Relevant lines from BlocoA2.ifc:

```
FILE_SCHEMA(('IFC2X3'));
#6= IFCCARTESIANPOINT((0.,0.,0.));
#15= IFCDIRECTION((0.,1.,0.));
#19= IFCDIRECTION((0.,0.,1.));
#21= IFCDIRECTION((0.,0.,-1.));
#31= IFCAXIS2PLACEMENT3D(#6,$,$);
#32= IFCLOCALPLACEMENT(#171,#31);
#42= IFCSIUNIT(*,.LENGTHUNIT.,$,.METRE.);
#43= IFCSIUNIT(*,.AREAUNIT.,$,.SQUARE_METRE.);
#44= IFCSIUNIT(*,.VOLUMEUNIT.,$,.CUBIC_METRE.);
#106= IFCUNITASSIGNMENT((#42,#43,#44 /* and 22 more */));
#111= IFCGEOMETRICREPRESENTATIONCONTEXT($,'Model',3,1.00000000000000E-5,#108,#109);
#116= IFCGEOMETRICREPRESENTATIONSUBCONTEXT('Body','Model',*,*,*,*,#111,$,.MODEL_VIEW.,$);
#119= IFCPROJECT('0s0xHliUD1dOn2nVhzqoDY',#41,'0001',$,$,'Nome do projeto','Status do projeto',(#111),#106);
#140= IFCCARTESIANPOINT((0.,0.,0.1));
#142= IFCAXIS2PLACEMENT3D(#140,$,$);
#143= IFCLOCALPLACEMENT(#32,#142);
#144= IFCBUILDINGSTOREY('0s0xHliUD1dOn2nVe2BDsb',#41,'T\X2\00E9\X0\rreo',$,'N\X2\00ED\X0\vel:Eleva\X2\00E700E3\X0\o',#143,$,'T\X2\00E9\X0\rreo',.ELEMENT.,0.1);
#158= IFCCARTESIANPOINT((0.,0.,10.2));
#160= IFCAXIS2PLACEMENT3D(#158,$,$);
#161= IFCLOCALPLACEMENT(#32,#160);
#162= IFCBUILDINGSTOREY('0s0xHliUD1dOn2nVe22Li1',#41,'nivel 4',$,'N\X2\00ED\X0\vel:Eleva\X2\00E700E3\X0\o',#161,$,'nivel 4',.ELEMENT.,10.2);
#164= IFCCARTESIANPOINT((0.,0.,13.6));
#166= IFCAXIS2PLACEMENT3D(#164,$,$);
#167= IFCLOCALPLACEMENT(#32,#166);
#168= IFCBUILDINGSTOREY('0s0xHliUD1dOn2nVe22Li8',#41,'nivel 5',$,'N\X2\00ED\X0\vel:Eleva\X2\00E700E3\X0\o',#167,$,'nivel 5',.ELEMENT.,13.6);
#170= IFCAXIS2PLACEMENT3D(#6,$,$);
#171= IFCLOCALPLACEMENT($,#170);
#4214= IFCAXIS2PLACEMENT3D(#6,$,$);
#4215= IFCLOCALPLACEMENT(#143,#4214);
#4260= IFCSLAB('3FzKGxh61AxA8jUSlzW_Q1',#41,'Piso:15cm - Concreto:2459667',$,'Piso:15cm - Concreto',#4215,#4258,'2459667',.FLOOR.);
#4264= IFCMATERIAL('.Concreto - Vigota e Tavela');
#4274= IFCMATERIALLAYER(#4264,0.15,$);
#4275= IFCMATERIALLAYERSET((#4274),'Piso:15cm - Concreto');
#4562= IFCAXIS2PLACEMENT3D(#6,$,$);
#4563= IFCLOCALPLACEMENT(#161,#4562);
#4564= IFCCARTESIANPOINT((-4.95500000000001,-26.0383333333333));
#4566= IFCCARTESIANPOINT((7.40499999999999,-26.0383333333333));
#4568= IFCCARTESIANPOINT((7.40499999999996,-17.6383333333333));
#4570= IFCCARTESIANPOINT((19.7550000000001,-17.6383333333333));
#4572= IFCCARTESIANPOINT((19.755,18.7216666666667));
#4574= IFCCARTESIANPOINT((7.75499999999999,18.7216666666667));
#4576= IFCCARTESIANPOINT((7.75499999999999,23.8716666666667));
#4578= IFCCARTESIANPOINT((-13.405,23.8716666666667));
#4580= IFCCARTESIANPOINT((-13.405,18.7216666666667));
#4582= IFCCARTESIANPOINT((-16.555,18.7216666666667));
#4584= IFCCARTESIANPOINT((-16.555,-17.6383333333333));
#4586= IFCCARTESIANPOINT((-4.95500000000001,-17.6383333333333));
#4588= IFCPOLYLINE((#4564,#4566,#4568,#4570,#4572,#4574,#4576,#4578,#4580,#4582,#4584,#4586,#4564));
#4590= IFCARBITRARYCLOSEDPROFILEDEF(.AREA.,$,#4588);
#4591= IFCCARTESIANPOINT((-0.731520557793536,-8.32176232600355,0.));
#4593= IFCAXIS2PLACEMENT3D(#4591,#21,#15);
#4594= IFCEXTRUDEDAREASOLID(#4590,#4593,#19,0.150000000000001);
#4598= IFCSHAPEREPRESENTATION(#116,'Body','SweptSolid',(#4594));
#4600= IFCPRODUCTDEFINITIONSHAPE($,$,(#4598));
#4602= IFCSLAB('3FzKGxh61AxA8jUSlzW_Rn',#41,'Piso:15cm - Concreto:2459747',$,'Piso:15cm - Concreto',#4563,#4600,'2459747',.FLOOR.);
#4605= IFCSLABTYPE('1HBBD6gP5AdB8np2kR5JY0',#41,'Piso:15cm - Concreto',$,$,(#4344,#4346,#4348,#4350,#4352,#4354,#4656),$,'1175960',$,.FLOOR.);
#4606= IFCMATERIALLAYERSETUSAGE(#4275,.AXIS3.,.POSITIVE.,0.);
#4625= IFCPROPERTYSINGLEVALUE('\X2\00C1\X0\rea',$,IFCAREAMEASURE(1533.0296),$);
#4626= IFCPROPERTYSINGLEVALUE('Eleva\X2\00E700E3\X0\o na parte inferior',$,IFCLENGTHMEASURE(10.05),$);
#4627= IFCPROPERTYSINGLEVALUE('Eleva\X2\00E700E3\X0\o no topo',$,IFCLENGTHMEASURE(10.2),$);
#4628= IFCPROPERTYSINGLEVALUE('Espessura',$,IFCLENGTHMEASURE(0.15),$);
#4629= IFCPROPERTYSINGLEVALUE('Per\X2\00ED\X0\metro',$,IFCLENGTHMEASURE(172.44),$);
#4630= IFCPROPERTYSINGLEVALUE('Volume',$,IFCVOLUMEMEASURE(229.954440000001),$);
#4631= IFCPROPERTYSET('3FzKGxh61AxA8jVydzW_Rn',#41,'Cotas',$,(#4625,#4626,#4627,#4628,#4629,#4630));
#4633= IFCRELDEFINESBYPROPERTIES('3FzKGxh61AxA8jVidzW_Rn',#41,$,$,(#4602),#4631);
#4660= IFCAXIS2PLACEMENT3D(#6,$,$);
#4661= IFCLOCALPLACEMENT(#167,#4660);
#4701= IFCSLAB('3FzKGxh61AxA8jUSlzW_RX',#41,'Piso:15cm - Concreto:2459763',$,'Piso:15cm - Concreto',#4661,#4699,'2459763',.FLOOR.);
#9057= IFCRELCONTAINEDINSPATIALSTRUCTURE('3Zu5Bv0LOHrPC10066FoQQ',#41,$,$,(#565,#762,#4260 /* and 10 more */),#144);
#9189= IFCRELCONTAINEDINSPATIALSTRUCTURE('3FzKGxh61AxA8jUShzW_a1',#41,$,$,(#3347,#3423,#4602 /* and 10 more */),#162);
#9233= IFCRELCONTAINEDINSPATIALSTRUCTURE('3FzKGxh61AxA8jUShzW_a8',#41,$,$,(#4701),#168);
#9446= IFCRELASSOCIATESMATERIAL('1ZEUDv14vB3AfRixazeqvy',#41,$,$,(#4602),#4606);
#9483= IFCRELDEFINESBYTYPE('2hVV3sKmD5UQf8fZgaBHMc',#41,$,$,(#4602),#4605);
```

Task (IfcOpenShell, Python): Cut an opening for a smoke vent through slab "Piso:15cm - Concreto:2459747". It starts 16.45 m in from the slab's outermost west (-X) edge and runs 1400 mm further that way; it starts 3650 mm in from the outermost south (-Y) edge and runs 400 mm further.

```python
import numpy as np
import ifcopenshell
import ifcopenshell.api.feature
import ifcopenshell.api.geometry
import ifcopenshell.api.pset
import ifcopenshell.api.root
import ifcopenshell.geom
import ifcopenshell.util.element
import ifcopenshell.util.placement
import ifcopenshell.util.representation
import ifcopenshell.util.shape
import ifcopenshell.util.unit

model = ifcopenshell.open("BlocoA2.ifc")
unit_scale = ifcopenshell.util.unit.calculate_unit_scale(model)
area_scale = ifcopenshell.util.unit.calculate_unit_scale(model, "AREAUNIT")
volume_scale = ifcopenshell.util.unit.calculate_unit_scale(model, "VOLUMEUNIT")
settings = ifcopenshell.geom.settings()


def volume(element):
    """Net volume in cubic metres, openings subtracted."""
    shape = ifcopenshell.geom.create_shape(settings, element)
    return ifcopenshell.util.shape.get_volume(shape.geometry)


slab = model.by_guid("3FzKGxh61AxA8jUSlzW_Rn")
before = volume(slab)

# Extent in the slab's own axes, in metres. The edges named are its -X and -Y sides.
slab_shape = ifcopenshell.geom.create_shape(settings, slab)
vertices = ifcopenshell.util.shape.get_vertices(slab_shape.geometry)
x_min, y_min, bottom = vertices.min(axis=0)
top = vertices[:, 2].max()

opening = ifcopenshell.api.root.create_entity(model, ifc_class="IfcOpeningElement", name="Smoke vent opening")
context = ifcopenshell.util.representation.get_context(model, "Model", "Body", "MODEL_VIEW")
width, depth = 1.4, 0.4
outline = [(0.0, 0.0), (width, 0.0), (width, depth), (0.0, depth), (0.0, 0.0)]
# Overshoot both faces by 50 mm so the cut is clean.
shape = ifcopenshell.api.geometry.add_slab_representation(
    model, context=context, depth=top - bottom + 0.1, polyline=outline
)
ifcopenshell.api.geometry.assign_representation(model, product=opening, representation=shape)

matrix = ifcopenshell.util.placement.get_local_placement(slab.ObjectPlacement)
matrix[:, 3] = matrix @ np.append(np.array([x_min + 16.45, y_min + 3.65, bottom - 0.05]) / unit_scale, 1.0)
ifcopenshell.api.geometry.edit_object_placement(model, product=opening, matrix=matrix, is_si=False)
ifcopenshell.api.feature.add_feature(model, feature=opening, element=slab)

after = volume(slab)

# Update the slab's stored quantities.
pset = model.by_id(ifcopenshell.util.element.get_pset(slab, "Cotas", should_inherit=False)["id"])
ifcopenshell.api.pset.edit_pset(model, pset=pset, properties={
    "Área": model.create_entity("IfcAreaMeasure", after / (top - bottom) / area_scale),
    "Volume": model.create_entity("IfcVolumeMeasure", after / volume_scale),
})

print(f"slab volume {before:.3f} -> {after:.3f} m3")

model.write("BlocoA2_rev.ifc")
```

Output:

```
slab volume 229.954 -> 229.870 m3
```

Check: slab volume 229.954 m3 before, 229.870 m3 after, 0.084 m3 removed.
